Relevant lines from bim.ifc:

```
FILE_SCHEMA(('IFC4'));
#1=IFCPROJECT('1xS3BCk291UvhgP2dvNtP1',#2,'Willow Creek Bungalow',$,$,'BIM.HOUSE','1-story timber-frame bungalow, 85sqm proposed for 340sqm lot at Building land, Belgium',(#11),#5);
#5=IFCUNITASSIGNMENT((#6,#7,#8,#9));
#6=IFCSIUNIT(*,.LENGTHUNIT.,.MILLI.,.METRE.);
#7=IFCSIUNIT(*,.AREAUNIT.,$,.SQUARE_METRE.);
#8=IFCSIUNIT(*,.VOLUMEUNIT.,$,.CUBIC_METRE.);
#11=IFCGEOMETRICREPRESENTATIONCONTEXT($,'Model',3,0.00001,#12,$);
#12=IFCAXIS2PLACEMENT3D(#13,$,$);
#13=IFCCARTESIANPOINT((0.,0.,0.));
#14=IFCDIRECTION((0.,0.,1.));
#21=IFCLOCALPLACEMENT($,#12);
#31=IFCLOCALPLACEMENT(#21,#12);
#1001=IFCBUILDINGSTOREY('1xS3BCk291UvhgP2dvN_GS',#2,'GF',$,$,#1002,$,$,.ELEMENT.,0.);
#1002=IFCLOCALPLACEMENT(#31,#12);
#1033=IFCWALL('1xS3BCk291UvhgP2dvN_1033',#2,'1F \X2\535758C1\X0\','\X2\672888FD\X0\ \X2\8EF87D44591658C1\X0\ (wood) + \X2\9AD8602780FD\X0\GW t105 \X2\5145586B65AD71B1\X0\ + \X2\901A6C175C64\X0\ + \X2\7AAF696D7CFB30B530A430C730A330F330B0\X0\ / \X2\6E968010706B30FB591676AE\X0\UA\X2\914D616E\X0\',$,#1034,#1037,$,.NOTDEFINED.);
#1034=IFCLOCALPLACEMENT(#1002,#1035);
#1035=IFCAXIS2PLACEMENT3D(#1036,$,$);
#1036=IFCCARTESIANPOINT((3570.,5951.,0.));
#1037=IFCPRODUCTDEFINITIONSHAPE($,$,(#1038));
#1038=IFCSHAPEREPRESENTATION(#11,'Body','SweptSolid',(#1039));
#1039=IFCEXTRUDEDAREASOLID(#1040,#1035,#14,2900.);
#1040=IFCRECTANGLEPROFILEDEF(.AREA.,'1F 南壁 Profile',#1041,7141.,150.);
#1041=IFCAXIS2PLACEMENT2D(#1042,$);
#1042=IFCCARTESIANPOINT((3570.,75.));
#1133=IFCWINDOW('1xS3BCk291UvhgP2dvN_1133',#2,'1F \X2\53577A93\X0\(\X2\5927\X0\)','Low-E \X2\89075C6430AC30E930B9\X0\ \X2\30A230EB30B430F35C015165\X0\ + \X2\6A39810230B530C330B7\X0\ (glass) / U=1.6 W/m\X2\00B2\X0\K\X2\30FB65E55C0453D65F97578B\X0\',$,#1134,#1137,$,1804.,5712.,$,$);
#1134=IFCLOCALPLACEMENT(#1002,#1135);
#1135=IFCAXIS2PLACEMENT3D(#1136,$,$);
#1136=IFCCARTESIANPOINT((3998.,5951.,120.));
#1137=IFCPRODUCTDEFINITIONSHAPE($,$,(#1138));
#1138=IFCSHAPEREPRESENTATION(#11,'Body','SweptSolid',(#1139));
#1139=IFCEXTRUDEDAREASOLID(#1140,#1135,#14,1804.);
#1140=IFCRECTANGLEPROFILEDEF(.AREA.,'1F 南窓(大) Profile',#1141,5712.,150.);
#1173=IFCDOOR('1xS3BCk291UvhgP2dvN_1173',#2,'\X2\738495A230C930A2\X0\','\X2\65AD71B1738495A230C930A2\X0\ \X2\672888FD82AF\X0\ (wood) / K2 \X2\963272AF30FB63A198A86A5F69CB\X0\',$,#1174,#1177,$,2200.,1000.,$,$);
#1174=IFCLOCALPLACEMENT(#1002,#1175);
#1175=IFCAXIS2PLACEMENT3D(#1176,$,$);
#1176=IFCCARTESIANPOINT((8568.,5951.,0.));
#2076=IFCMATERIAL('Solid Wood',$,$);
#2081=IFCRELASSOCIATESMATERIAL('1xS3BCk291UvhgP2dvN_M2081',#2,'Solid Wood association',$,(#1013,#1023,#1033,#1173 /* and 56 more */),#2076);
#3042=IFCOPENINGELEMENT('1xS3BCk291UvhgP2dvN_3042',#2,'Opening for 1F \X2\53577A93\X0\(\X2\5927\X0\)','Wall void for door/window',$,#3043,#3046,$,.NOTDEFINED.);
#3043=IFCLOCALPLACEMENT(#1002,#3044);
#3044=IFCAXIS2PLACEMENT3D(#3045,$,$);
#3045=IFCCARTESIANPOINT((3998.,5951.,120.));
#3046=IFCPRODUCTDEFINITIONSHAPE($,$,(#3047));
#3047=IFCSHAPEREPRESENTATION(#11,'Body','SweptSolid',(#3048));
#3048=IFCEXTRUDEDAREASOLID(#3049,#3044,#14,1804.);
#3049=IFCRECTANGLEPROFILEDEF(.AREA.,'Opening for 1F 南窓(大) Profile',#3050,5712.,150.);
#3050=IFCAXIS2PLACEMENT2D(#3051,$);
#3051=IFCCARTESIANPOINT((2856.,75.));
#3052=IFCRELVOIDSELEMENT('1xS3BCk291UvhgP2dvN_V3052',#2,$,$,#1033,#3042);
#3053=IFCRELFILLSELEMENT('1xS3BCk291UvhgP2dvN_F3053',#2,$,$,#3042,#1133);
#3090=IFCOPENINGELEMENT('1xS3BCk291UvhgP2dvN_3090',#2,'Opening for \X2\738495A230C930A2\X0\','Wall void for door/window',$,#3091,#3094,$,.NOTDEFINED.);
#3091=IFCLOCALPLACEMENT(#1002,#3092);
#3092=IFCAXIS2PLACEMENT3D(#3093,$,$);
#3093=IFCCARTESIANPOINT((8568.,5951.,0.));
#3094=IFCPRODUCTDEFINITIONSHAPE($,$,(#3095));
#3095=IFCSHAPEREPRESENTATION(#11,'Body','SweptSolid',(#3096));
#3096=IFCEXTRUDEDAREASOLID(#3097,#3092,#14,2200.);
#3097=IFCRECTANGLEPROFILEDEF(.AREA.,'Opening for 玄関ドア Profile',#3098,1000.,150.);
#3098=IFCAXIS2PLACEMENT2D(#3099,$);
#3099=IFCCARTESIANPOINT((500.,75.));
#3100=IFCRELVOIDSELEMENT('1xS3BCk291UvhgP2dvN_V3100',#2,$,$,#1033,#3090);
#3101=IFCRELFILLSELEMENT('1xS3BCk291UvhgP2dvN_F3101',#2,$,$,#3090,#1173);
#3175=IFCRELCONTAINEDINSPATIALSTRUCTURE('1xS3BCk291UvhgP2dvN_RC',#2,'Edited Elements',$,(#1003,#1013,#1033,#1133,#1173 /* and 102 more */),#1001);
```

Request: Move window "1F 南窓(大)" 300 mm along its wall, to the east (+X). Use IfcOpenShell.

```python
import ifcopenshell
import ifcopenshell.api.geometry
import ifcopenshell.util.placement

model = ifcopenshell.open("bim.ifc")

window = model.by_id(1133)
opening = window.FillsVoids[0].RelatingOpeningElement
wall = opening.VoidsElements[0].RelatingBuildingElement

wall_matrix = ifcopenshell.util.placement.get_local_placement(wall.ObjectPlacement)
shift = wall_matrix[:3, 0] * 300.0
before = ifcopenshell.util.placement.get_local_placement(window.ObjectPlacement)[:3, 3].copy()

# The window is not placed relative to its opening, so move both.
for product in (opening, window):
    matrix = ifcopenshell.util.placement.get_local_placement(product.ObjectPlacement)
    matrix[:3, 3] += shift
    ifcopenshell.api.geometry.edit_object_placement(model, product=product, matrix=matrix, is_si=False)

after = ifcopenshell.util.placement.get_local_placement(window.ObjectPlacement)[:3, 3]
print("window moved by", (after - before).round(3) + 0.0)

model.write("bim_edited.ifc")
```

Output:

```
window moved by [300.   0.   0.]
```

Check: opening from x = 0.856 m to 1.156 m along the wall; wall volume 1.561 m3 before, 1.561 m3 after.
